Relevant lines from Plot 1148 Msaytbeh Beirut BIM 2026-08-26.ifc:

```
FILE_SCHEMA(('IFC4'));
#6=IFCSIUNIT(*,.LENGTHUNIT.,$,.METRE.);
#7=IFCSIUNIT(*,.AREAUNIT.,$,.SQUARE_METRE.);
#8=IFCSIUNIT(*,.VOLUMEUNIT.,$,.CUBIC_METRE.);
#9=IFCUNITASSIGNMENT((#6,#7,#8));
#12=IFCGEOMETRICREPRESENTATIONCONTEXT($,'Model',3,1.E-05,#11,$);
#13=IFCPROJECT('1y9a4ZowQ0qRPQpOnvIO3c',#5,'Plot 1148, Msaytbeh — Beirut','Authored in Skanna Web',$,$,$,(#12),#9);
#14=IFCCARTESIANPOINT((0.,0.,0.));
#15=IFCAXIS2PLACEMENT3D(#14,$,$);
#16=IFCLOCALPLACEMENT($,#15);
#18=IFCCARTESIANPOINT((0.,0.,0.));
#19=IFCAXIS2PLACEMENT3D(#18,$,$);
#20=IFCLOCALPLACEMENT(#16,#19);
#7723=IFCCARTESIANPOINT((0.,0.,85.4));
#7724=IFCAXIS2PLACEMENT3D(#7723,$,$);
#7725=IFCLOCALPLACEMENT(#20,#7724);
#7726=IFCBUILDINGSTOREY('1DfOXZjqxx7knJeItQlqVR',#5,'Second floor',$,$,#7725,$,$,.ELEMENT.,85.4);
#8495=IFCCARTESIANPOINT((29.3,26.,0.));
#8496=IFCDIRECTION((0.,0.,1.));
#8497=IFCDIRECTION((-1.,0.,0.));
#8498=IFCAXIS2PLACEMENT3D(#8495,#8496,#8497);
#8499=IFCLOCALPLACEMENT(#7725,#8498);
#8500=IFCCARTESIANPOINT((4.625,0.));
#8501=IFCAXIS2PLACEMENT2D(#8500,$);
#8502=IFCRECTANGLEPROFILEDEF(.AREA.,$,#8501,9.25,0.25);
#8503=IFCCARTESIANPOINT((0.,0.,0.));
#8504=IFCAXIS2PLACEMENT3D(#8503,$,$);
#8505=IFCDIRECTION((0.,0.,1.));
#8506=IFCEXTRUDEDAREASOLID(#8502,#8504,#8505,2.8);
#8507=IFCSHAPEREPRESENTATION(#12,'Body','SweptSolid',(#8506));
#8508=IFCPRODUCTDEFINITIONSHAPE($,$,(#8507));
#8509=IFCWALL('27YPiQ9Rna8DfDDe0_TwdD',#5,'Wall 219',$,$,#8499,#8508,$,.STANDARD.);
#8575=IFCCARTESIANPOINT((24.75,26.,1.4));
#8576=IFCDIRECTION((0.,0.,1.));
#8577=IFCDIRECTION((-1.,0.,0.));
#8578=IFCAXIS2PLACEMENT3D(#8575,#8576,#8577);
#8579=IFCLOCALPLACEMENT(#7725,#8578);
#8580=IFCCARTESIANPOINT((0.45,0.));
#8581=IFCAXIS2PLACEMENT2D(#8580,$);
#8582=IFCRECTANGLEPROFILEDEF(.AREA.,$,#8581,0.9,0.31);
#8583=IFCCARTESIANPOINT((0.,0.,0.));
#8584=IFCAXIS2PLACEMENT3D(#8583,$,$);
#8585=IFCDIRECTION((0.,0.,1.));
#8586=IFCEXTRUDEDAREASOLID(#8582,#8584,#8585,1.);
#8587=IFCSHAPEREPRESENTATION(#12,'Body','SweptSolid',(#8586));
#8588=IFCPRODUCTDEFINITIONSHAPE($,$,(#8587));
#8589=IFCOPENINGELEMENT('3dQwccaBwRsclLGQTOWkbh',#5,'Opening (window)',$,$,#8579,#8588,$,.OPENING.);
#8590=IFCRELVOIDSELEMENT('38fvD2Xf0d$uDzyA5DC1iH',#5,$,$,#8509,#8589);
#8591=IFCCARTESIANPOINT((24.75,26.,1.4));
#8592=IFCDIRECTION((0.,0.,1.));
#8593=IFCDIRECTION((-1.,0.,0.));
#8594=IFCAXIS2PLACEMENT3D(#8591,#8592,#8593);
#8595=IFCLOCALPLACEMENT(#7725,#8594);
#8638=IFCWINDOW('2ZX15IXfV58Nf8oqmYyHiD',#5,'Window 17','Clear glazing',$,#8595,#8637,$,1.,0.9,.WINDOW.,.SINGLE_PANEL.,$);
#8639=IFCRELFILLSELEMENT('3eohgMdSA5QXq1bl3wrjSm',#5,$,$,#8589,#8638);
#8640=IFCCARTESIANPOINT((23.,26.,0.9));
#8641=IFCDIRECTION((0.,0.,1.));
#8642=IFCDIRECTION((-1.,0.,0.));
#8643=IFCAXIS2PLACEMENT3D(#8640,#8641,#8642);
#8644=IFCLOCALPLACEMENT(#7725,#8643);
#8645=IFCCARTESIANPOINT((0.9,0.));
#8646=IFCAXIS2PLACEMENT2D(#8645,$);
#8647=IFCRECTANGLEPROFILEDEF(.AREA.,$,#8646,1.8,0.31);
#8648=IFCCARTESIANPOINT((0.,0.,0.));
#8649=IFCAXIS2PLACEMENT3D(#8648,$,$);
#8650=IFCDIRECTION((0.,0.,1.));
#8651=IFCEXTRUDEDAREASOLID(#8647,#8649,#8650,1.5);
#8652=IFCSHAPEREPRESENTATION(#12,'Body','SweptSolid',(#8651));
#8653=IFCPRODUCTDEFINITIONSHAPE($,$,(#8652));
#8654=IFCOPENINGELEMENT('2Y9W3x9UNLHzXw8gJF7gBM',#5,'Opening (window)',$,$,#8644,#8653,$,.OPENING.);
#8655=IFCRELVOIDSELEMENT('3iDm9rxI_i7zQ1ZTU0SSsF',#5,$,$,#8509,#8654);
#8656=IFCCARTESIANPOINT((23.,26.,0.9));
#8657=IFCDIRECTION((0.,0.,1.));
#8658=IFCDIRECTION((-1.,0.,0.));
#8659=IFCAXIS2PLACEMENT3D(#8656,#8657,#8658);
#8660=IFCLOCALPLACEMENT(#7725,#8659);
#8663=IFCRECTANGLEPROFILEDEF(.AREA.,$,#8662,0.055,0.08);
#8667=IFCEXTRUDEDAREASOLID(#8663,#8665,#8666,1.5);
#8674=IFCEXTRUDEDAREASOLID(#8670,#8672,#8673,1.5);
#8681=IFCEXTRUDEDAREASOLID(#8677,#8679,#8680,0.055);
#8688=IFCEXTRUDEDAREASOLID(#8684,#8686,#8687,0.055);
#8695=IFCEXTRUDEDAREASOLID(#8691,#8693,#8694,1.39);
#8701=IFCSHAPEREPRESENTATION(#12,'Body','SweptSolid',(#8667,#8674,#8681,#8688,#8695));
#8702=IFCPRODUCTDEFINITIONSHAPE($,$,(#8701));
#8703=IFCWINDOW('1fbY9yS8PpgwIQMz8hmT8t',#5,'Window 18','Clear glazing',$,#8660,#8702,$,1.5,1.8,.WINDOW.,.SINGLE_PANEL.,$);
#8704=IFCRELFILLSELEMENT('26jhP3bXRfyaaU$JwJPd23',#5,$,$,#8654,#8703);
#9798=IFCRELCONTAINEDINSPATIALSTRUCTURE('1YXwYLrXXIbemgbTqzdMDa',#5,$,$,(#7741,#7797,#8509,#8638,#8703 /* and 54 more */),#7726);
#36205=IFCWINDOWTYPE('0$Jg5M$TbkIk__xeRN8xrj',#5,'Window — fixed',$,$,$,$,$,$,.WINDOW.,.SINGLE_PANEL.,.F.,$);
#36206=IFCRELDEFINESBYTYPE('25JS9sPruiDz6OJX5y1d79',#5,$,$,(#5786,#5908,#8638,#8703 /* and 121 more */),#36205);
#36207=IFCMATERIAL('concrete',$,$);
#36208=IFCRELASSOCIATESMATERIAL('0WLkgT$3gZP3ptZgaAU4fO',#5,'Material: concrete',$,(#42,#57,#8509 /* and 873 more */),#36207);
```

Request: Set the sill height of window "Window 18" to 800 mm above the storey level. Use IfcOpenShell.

```python
import numpy as np
import ifcopenshell
import ifcopenshell.api.geometry
import ifcopenshell.geom
import ifcopenshell.util.element
import ifcopenshell.util.placement
import ifcopenshell.util.shape
import ifcopenshell.util.unit

model = ifcopenshell.open("Plot 1148 Msaytbeh Beirut BIM 2026-08-26.ifc")
unit_scale = ifcopenshell.util.unit.calculate_unit_scale(model)

window = model.by_guid("1fbY9yS8PpgwIQMz8hmT8t")
opening = window.FillsVoids[0].RelatingOpeningElement
storey = ifcopenshell.util.element.get_container(window, ifc_class="IfcBuildingStorey")
level = ifcopenshell.util.placement.get_local_placement(storey.ObjectPlacement)[2, 3]

# The opening's origin need not be at the sill, so measure its lowest point.
shape = ifcopenshell.geom.create_shape(ifcopenshell.geom.settings(), opening)
bottom = ifcopenshell.util.shape.get_shape_bottom_elevation(shape, shape.geometry) / unit_scale
dz = level + 0.8 - bottom

shift = np.array([0.0, 0.0, dz])
# The window is not placed relative to its opening, so move both.
for product in (opening, window):
    matrix = ifcopenshell.util.placement.get_local_placement(product.ObjectPlacement)
    matrix[:3, 3] += shift
    ifcopenshell.api.geometry.edit_object_placement(model, product=product, matrix=matrix, is_si=False)

print(f"moved by {dz * unit_scale:+.3f} m")

model.write("Plot 1148 Msaytbeh Beirut BIM 2026-08-26_edited.ifc")
```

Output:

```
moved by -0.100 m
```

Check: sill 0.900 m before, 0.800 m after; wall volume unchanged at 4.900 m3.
